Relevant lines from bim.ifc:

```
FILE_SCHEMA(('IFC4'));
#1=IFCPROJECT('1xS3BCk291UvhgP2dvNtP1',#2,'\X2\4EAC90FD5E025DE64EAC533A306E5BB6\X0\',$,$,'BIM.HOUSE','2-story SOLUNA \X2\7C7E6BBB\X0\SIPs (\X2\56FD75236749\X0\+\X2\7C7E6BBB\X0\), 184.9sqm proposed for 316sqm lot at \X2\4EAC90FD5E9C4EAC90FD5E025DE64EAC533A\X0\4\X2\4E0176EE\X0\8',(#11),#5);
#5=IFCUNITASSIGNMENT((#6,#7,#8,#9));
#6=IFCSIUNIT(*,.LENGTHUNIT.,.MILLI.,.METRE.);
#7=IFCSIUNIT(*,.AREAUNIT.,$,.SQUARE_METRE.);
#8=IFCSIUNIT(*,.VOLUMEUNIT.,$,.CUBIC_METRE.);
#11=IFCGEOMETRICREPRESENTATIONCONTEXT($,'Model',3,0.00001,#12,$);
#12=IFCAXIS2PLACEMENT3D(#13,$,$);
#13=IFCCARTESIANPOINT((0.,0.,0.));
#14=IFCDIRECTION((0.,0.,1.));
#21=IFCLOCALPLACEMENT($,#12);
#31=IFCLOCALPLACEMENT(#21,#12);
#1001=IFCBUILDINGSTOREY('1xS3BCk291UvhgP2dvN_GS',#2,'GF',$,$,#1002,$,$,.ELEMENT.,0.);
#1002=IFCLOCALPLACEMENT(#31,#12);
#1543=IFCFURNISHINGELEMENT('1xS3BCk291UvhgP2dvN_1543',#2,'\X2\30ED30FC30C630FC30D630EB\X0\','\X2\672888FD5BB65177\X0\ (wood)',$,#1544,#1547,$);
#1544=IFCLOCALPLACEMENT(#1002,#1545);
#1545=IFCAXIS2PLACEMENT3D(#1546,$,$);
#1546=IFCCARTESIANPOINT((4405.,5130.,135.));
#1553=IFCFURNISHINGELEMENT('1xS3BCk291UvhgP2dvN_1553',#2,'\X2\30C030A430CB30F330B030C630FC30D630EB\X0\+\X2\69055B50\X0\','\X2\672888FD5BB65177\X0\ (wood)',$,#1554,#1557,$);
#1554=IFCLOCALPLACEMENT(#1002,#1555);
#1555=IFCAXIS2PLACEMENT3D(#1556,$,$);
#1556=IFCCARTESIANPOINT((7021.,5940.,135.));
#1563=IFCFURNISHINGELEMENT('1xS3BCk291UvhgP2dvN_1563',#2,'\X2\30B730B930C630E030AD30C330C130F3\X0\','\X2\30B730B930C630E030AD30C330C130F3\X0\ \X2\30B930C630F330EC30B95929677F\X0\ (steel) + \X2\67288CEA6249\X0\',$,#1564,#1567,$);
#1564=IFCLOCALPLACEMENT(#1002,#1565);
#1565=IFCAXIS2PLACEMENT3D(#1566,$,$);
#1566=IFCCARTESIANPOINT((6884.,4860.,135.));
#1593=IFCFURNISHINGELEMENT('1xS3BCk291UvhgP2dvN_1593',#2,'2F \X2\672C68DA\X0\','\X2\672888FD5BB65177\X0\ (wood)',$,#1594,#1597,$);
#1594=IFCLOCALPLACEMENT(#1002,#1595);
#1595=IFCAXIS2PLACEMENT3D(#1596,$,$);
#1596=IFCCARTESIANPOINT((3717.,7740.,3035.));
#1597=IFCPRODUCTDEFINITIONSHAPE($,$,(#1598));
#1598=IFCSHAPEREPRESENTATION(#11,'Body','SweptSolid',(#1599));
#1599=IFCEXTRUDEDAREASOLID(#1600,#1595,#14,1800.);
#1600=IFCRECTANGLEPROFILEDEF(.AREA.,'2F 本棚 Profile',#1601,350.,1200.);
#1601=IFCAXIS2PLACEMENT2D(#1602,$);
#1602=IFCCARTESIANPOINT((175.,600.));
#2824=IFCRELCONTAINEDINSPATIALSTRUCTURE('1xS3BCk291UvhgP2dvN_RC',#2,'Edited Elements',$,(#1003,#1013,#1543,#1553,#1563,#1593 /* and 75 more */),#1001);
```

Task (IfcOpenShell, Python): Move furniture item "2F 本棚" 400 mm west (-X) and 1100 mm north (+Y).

```python
import ifcopenshell
import ifcopenshell.api.geometry
import ifcopenshell.util.placement
import ifcopenshell.util.unit

model = ifcopenshell.open("bim.ifc")
unit_scale = ifcopenshell.util.unit.calculate_unit_scale(model)

item = model.by_guid("1xS3BCk291UvhgP2dvN_1593")
matrix = ifcopenshell.util.placement.get_local_placement(item.ObjectPlacement)
matrix[0, 3] -= 0.4 / unit_scale
matrix[1, 3] += 1.1 / unit_scale
ifcopenshell.api.geometry.edit_object_placement(model, product=item, matrix=matrix, is_si=False)

print(ifcopenshell.util.placement.get_local_placement(item.ObjectPlacement).round(3) + 0.0)

model.write("bim_edited.ifc")
```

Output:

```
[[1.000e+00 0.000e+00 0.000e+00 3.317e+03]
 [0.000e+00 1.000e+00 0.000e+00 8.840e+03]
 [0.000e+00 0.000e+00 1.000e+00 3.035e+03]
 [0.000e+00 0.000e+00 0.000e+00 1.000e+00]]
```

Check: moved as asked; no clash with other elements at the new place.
